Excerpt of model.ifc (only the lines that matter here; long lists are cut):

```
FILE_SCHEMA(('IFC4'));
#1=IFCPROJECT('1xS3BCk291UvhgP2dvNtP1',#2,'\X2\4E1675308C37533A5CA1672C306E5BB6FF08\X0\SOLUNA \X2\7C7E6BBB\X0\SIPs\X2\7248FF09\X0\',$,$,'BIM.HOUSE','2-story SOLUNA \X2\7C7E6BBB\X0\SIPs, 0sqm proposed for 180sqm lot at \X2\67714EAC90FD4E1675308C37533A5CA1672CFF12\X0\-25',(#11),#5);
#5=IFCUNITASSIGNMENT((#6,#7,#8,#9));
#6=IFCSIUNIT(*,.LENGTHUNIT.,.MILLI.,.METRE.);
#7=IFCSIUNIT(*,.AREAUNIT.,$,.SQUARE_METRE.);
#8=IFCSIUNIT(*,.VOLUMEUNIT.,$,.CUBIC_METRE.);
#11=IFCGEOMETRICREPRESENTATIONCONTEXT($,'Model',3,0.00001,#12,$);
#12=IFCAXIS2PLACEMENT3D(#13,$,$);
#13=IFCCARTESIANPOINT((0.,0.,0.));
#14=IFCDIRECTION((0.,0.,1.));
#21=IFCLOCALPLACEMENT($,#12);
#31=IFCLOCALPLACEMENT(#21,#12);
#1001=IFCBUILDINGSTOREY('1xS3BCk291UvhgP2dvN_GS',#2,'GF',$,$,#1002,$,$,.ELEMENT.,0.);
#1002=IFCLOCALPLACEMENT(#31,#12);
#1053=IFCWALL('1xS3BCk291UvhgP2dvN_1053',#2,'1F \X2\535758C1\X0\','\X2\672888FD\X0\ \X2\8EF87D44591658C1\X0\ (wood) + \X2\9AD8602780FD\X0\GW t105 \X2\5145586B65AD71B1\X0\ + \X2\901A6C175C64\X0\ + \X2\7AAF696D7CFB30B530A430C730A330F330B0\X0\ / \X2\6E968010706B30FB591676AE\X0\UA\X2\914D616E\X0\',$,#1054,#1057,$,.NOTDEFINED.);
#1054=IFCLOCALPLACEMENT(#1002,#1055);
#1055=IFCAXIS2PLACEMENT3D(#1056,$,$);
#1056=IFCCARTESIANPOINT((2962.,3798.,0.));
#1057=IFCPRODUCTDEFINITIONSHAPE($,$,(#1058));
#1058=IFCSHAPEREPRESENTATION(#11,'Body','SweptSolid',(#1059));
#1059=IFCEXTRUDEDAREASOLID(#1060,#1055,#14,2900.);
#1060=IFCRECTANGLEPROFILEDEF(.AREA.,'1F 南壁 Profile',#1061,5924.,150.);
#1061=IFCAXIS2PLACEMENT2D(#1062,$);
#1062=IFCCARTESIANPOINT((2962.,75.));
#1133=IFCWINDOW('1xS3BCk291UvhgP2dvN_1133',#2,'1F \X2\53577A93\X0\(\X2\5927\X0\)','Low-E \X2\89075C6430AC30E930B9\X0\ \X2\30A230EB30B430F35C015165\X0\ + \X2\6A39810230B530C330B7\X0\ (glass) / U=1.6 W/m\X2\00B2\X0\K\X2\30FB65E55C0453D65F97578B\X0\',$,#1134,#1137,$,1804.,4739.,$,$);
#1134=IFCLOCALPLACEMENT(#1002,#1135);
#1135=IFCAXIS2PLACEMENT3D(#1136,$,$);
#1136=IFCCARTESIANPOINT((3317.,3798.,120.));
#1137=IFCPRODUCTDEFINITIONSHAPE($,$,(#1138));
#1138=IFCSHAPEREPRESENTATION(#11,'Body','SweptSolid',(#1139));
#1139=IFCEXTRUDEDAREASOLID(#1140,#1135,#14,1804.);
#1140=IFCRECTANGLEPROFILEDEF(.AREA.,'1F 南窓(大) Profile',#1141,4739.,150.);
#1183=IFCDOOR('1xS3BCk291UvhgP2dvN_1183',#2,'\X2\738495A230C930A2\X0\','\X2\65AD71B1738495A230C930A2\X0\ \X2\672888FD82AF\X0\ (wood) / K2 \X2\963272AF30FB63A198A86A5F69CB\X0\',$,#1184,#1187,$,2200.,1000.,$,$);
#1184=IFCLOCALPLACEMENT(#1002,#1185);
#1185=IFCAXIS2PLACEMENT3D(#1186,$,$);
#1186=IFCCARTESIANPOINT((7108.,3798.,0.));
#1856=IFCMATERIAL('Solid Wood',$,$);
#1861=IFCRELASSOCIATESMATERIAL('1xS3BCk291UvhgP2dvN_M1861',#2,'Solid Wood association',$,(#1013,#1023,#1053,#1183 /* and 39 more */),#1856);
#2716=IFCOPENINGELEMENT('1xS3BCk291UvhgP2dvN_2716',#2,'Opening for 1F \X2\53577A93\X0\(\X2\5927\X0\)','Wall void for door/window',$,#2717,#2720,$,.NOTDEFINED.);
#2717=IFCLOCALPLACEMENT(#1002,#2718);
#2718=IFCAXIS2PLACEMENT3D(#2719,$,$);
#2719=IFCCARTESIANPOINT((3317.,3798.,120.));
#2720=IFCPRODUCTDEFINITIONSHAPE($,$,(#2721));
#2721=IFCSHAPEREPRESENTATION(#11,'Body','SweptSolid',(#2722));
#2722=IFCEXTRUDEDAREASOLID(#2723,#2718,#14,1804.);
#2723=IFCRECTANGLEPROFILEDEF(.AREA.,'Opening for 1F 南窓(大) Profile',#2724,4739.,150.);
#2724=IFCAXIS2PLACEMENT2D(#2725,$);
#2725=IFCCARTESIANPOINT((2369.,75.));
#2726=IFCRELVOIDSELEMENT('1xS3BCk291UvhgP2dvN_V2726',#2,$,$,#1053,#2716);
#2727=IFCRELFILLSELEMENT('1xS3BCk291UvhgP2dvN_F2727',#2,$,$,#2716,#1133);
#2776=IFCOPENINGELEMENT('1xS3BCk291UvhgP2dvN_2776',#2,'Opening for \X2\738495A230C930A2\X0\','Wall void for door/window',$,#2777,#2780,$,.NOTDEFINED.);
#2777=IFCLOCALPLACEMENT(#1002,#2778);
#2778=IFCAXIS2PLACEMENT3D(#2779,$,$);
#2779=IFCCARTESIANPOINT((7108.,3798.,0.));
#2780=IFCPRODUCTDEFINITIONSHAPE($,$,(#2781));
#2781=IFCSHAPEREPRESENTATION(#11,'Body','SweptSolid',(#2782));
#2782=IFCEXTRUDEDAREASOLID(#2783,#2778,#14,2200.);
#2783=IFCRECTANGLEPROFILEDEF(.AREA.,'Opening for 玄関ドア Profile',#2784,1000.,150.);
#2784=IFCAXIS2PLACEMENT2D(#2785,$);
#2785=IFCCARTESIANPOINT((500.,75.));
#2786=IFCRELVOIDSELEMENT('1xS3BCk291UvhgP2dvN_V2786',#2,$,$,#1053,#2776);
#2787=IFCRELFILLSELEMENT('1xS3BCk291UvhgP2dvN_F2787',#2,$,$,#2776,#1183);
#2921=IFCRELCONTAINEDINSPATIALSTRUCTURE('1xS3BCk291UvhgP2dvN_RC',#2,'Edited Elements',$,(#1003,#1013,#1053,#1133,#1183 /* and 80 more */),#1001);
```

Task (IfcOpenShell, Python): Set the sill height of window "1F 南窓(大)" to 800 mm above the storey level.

```python
import numpy as np
import ifcopenshell
import ifcopenshell.api.geometry
import ifcopenshell.geom
import ifcopenshell.util.element
import ifcopenshell.util.placement
import ifcopenshell.util.shape
import ifcopenshell.util.unit

model = ifcopenshell.open("model.ifc")
unit_scale = ifcopenshell.util.unit.calculate_unit_scale(model)

window = model.by_id(1133)
opening = window.FillsVoids[0].RelatingOpeningElement
storey = ifcopenshell.util.element.get_container(window, ifc_class="IfcBuildingStorey")
level = ifcopenshell.util.placement.get_local_placement(storey.ObjectPlacement)[2, 3]

# The opening's origin need not be at the sill, so measure its lowest point.
shape = ifcopenshell.geom.create_shape(ifcopenshell.geom.settings(), opening)
bottom = ifcopenshell.util.shape.get_shape_bottom_elevation(shape, shape.geometry) / unit_scale
dz = level + 0.8 / unit_scale - bottom

shift = np.array([0.0, 0.0, dz])
# The window is not placed relative to its opening, so move both.
for product in (opening, window):
    matrix = ifcopenshell.util.placement.get_local_placement(product.ObjectPlacement)
    matrix[:3, 3] += shift
    ifcopenshell.api.geometry.edit_object_placement(model, product=product, matrix=matrix, is_si=False)

print(f"moved by {dz * unit_scale:+.3f} m")

model.write("model_edited.ifc")
```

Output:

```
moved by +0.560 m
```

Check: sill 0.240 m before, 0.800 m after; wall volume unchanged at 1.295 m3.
